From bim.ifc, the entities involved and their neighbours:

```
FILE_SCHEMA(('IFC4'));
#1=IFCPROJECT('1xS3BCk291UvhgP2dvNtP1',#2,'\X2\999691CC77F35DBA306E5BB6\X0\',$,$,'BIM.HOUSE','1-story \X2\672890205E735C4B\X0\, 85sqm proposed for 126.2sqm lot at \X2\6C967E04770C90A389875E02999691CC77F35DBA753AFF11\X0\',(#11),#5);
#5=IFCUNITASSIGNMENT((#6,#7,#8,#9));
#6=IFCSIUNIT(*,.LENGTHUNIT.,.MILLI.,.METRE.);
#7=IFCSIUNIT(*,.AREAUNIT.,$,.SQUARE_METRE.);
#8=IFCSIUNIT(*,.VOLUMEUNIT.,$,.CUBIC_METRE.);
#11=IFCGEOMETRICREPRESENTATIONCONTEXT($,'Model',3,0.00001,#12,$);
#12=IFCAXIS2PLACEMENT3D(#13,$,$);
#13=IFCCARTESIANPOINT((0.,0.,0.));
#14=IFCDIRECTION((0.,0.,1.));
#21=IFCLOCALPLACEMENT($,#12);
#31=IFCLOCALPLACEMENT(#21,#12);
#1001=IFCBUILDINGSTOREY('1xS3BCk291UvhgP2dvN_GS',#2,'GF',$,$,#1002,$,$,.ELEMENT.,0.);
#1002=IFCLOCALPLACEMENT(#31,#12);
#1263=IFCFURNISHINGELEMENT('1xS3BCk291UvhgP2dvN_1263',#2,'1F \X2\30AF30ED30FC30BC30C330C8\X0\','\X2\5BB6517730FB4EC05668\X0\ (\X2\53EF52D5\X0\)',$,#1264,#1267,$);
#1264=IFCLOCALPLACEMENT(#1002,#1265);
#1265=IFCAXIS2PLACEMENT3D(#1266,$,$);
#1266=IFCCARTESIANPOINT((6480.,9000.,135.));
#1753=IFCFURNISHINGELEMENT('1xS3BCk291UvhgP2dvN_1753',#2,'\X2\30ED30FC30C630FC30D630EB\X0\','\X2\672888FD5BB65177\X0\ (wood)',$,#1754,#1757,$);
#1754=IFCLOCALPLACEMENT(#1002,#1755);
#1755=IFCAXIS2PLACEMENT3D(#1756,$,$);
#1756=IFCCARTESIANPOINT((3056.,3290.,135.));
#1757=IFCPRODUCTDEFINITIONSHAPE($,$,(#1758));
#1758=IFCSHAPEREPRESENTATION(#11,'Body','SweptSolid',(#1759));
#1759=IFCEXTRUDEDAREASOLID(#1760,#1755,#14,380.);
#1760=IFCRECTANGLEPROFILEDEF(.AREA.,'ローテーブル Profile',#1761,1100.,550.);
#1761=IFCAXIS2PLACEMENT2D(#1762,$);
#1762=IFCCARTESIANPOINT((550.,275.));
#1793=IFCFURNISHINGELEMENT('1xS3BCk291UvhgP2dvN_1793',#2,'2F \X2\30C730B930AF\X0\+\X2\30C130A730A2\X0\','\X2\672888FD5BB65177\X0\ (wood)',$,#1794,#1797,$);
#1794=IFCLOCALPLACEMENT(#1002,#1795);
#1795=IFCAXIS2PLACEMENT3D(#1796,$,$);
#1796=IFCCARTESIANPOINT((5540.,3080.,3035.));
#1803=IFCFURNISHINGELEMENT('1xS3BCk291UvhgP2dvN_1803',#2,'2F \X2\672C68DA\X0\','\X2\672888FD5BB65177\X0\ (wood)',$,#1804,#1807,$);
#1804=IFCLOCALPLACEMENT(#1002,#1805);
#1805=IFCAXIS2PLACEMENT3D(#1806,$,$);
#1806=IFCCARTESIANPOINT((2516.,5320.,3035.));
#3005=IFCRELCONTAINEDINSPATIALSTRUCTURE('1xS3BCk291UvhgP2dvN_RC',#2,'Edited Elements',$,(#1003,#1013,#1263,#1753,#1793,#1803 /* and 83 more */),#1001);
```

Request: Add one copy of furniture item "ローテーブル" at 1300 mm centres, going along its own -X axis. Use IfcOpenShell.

```python
import ifcopenshell
import ifcopenshell.api.geometry
import ifcopenshell.api.root
import ifcopenshell.util.element
import ifcopenshell.util.placement
import ifcopenshell.util.unit

model = ifcopenshell.open("bim.ifc")
unit_scale = ifcopenshell.util.unit.calculate_unit_scale(model)


def reuse_history(source, copy):
    """copy_class also copies each property set's owner history, people and application; keep the originals."""
    for rel in copy.IsDefinedBy:
        if rel.is_a("IfcRelDefinesByProperties") and (history := rel.RelatingPropertyDefinition.OwnerHistory):
            rel.RelatingPropertyDefinition.OwnerHistory = source.OwnerHistory
            ifcopenshell.util.element.remove_deep2(model, history)


source = model.by_guid("1xS3BCk291UvhgP2dvN_1753")
base = ifcopenshell.util.placement.get_local_placement(source.ObjectPlacement)
step = -base[:3, 0] * 1.3 / unit_scale

for i in range(1, 2):
    copy = ifcopenshell.api.root.copy_class(model, product=source)
    copy.Representation = ifcopenshell.util.element.copy_deep(
        model, source.Representation, exclude=["IfcGeometricRepresentationContext", "IfcRepresentationMap"]
    )
    reuse_history(source, copy)
    matrix = base.copy()
    matrix[:3, 3] += i * step
    print("added at", matrix[:3, 3].round(3) + 0.0)
    ifcopenshell.api.geometry.edit_object_placement(model, product=copy, matrix=matrix, is_si=False)

model.write("bim_edited.ifc")
```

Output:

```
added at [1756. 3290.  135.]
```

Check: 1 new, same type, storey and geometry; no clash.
